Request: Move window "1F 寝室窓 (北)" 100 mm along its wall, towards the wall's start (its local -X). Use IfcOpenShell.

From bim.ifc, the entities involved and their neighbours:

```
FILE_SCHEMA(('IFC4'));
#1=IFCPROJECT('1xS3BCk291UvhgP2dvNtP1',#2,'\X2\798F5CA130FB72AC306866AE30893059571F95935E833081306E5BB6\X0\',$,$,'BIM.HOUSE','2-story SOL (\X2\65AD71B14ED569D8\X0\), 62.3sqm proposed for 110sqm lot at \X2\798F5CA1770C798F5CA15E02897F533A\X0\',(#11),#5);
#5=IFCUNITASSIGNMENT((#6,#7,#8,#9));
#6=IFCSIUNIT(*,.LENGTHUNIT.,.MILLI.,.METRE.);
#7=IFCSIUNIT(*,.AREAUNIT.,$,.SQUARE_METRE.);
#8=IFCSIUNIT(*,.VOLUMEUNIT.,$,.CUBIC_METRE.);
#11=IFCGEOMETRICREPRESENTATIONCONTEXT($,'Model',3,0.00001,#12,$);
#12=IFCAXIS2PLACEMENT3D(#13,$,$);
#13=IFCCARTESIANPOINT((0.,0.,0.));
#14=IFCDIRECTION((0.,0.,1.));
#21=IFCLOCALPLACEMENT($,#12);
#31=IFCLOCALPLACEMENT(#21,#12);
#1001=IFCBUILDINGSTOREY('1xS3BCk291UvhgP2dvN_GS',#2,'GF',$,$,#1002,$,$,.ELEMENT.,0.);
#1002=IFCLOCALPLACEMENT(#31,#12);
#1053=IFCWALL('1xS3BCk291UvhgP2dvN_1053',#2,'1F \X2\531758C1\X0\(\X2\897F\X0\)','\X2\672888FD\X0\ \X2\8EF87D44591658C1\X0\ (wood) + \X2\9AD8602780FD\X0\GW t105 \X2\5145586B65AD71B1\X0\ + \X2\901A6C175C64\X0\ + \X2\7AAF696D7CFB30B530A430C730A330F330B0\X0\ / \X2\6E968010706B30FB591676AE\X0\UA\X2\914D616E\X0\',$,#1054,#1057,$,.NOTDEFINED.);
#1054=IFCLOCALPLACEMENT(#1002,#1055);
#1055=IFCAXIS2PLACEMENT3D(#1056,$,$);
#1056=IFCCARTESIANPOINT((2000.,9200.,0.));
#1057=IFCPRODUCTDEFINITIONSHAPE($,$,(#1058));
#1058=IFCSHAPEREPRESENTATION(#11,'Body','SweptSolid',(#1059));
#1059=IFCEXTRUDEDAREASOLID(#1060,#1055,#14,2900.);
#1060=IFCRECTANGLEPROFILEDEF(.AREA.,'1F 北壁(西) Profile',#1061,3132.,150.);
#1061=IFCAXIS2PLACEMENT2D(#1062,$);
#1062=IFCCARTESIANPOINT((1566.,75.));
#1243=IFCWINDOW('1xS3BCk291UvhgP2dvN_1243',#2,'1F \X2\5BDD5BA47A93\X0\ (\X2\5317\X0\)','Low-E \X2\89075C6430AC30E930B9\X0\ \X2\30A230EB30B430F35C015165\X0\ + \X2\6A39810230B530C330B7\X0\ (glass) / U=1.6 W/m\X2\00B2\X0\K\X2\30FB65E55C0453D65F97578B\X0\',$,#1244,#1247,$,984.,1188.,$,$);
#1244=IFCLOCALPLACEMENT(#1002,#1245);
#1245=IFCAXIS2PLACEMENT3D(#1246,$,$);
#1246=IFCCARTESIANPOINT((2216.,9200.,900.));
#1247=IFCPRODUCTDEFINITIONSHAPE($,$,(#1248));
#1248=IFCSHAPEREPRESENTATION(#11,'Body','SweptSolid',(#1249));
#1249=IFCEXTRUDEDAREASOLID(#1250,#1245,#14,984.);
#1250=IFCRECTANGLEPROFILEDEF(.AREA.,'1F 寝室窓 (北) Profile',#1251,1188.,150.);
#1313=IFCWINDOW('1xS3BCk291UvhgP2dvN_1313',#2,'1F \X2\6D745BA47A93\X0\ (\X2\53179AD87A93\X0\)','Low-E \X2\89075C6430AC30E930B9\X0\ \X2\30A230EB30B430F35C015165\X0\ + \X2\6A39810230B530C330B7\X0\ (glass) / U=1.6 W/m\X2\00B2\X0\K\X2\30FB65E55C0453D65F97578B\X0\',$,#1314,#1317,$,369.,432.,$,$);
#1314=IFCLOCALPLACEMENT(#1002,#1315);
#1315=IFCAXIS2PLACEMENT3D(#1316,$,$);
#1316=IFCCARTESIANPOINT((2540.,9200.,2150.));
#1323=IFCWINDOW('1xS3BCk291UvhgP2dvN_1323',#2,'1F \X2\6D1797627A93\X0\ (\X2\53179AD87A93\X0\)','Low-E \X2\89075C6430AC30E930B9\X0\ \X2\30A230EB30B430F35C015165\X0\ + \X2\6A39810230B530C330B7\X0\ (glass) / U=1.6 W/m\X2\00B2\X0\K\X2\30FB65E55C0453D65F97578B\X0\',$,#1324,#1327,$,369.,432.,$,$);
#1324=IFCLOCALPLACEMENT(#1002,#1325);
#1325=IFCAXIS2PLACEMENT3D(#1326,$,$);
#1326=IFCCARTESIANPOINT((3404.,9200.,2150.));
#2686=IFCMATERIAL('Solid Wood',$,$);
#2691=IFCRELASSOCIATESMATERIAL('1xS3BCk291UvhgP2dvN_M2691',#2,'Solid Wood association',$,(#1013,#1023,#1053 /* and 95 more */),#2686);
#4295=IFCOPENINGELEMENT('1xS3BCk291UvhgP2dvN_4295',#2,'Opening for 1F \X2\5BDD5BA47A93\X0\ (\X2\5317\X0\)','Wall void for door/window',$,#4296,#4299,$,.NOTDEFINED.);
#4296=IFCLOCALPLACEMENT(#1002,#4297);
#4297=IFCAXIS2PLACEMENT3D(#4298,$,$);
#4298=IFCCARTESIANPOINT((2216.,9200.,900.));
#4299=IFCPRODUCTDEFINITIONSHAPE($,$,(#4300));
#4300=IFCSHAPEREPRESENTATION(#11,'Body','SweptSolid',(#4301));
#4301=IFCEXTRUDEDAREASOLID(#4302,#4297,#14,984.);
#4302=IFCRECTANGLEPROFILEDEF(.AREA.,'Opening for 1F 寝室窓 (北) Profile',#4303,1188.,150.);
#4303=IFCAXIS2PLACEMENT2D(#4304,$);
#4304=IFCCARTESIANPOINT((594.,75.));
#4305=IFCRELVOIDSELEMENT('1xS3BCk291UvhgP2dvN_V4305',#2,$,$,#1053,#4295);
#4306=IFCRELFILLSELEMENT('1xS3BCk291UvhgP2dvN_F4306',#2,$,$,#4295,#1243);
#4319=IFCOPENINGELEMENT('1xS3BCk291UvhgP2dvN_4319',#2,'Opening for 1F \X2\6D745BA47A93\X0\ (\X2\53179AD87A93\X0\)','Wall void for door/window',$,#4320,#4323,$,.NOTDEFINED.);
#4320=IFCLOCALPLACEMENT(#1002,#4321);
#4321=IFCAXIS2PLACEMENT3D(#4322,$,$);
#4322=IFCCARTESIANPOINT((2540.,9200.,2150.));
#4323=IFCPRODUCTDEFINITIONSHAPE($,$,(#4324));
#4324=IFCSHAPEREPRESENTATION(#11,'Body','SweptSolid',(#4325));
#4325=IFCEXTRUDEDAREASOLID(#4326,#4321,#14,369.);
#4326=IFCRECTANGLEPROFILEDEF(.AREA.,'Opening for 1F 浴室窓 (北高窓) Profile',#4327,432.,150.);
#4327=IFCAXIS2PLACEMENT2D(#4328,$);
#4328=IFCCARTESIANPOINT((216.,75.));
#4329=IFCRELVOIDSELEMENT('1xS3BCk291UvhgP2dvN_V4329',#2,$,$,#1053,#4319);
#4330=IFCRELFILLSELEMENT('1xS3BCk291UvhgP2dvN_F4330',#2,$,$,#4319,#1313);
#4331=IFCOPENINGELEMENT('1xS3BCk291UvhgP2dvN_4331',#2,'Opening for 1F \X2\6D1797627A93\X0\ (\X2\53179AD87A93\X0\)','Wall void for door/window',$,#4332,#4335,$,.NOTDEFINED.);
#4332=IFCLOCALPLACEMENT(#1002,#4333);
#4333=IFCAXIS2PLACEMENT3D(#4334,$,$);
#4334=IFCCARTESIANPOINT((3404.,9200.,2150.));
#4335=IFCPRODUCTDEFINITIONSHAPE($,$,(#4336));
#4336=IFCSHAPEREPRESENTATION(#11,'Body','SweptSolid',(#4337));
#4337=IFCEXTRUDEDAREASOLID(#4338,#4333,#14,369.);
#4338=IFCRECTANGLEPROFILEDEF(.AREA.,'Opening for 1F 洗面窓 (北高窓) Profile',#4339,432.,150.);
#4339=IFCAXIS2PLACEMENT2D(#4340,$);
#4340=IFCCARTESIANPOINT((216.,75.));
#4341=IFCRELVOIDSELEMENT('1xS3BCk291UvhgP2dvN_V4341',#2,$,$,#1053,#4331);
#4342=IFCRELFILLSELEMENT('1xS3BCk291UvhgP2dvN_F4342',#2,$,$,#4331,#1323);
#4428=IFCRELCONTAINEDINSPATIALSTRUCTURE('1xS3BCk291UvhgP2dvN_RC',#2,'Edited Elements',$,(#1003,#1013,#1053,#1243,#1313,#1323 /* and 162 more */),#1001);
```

```python
import ifcopenshell
import ifcopenshell.api.geometry
import ifcopenshell.util.placement

model = ifcopenshell.open("bim.ifc")

window = model.by_id(1243)
opening = window.FillsVoids[0].RelatingOpeningElement
wall = opening.VoidsElements[0].RelatingBuildingElement

wall_matrix = ifcopenshell.util.placement.get_local_placement(wall.ObjectPlacement)
shift = wall_matrix[:3, 0] * -100.0
before = ifcopenshell.util.placement.get_local_placement(window.ObjectPlacement)[:3, 3].copy()

# The window is not placed relative to its opening, so move both.
for product in (opening, window):
    matrix = ifcopenshell.util.placement.get_local_placement(product.ObjectPlacement)
    matrix[:3, 3] += shift
    ifcopenshell.api.geometry.edit_object_placement(model, product=product, matrix=matrix, is_si=False)

after = ifcopenshell.util.placement.get_local_placement(window.ObjectPlacement)[:3, 3]
print("window moved by", (after - before).round(3) + 0.0)

model.write("bim_v2.ifc")
```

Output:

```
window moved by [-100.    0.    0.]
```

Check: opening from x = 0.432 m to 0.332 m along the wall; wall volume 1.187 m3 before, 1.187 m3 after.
